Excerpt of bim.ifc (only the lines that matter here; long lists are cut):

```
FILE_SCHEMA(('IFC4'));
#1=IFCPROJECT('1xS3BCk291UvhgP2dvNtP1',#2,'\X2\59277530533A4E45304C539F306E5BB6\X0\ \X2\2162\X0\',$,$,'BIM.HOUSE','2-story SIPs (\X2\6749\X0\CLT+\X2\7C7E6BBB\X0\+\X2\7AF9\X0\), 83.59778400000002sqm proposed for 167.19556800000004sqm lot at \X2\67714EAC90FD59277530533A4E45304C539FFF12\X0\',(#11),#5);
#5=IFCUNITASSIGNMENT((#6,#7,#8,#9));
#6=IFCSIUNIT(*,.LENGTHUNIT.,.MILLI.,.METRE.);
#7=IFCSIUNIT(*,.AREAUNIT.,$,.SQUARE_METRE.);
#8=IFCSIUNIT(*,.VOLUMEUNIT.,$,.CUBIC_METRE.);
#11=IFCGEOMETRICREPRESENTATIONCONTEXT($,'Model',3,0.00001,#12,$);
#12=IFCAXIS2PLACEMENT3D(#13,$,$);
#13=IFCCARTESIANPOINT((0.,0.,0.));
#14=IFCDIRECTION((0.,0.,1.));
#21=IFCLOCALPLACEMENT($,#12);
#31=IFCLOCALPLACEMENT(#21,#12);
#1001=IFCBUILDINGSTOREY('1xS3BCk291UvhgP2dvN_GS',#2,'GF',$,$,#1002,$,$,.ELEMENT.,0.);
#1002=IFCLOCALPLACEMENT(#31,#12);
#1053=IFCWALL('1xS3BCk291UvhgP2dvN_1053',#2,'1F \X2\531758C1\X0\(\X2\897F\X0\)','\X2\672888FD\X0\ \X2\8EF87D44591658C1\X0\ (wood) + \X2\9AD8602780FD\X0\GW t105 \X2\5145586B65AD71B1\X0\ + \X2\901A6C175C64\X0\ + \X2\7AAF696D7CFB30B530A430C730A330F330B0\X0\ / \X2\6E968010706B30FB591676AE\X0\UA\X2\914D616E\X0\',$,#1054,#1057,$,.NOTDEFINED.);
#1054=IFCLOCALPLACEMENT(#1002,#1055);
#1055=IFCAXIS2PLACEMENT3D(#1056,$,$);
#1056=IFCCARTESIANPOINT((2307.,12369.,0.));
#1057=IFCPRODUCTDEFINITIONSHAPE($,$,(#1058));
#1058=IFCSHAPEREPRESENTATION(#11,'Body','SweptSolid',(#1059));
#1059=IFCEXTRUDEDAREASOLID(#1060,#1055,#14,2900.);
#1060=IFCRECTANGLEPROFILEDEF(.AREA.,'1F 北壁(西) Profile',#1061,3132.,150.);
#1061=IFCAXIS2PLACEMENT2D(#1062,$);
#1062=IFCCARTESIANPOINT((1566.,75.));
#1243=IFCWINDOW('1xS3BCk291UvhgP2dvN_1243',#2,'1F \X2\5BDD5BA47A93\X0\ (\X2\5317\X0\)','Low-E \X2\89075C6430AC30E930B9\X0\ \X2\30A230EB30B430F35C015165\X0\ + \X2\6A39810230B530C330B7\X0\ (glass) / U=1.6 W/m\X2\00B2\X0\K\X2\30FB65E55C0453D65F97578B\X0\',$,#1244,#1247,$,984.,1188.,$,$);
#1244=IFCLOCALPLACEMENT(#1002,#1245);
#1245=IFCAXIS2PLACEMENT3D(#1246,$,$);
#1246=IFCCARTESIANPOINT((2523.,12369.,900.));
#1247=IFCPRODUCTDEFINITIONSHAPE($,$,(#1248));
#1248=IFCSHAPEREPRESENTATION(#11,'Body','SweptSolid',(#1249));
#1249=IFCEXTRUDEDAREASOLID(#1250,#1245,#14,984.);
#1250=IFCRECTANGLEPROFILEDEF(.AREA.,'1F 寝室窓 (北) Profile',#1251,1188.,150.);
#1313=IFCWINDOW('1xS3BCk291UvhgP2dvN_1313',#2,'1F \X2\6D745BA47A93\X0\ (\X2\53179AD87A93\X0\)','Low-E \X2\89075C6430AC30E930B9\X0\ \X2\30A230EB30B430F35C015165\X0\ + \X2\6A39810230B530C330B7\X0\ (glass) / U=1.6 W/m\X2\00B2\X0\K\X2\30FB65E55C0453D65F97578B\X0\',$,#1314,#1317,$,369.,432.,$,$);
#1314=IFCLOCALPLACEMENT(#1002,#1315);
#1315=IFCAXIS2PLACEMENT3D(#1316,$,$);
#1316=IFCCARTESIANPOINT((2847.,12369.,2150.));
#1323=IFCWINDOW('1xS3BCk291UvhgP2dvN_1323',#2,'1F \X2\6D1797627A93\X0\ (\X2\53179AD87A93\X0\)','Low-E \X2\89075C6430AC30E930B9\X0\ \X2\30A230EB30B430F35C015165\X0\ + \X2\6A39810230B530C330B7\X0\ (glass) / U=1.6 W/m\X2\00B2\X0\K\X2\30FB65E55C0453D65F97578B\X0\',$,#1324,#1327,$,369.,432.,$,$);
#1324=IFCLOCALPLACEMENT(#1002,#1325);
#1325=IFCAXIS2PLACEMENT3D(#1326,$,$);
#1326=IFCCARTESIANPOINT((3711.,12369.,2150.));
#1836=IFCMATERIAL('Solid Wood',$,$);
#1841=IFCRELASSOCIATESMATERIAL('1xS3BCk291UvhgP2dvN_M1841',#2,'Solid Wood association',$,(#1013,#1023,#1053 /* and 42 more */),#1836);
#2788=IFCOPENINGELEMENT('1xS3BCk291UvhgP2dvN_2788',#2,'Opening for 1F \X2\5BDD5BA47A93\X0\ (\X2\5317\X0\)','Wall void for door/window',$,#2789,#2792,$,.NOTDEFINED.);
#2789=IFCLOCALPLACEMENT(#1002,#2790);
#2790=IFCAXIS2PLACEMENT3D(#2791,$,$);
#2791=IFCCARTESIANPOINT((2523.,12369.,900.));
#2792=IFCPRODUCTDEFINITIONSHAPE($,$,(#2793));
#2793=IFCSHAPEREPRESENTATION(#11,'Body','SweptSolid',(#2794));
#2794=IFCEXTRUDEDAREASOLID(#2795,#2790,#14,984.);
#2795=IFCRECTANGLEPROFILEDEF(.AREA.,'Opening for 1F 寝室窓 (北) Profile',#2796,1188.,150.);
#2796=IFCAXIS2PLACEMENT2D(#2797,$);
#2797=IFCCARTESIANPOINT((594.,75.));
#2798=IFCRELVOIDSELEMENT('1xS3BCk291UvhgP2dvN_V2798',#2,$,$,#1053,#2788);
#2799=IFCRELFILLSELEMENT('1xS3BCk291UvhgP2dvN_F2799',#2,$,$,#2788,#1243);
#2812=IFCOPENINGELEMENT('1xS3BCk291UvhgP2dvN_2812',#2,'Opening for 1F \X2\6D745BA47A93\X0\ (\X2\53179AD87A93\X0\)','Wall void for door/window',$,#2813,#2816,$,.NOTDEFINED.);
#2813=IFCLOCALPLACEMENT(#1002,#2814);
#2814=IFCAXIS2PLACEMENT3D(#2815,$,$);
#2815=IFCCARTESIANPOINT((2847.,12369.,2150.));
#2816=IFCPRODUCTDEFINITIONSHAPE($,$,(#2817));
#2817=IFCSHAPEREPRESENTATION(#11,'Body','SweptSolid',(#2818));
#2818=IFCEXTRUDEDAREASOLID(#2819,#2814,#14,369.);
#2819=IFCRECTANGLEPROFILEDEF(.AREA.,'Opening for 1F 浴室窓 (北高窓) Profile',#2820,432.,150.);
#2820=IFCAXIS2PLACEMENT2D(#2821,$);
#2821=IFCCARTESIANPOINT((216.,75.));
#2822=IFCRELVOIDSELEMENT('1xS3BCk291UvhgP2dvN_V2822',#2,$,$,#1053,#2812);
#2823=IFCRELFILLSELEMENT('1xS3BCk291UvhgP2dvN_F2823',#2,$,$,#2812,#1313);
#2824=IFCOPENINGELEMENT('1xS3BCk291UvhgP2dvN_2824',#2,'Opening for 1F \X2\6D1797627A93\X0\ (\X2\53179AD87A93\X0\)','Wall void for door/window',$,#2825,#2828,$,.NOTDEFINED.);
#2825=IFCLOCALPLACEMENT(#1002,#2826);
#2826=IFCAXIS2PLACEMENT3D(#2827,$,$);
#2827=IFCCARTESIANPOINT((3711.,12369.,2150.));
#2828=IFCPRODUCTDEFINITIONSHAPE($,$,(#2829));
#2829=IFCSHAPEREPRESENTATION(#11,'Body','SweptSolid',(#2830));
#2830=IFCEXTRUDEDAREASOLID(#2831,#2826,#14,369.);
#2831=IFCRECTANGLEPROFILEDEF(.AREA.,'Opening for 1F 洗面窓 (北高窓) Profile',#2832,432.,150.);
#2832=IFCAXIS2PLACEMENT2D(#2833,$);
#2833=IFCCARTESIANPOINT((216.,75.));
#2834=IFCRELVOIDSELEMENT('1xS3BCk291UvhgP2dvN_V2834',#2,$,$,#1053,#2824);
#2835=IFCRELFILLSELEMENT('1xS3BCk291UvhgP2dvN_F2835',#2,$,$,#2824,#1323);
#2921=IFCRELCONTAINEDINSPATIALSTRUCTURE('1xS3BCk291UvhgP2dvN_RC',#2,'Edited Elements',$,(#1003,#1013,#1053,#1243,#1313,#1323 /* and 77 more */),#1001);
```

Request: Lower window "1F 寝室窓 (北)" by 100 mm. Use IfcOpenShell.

```python
import numpy as np
import ifcopenshell
import ifcopenshell.api.geometry
import ifcopenshell.util.placement
import ifcopenshell.util.unit

model = ifcopenshell.open("bim.ifc")
unit_scale = ifcopenshell.util.unit.calculate_unit_scale(model)

window = model.by_guid("1xS3BCk291UvhgP2dvN_1243")
opening = window.FillsVoids[0].RelatingOpeningElement
dz = -0.1 / unit_scale

shift = np.array([0.0, 0.0, dz])
# The window is not placed relative to its opening, so move both.
for product in (opening, window):
    matrix = ifcopenshell.util.placement.get_local_placement(product.ObjectPlacement)
    matrix[:3, 3] += shift
    ifcopenshell.api.geometry.edit_object_placement(model, product=product, matrix=matrix, is_si=False)

print(f"moved by {dz * unit_scale:+.3f} m")

model.write("bim_updated.ifc")
```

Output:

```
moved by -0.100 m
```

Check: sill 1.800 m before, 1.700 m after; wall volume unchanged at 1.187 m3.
